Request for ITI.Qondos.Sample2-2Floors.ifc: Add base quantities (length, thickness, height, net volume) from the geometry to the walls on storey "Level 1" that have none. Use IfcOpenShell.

First a look at what the model holds.

```python
import ifcopenshell
import ifcopenshell.util.element
import ifcopenshell.util.unit

model = ifcopenshell.open("ITI.Qondos.Sample2-2Floors.ifc")
print(model.schema)
for unit_type in ("LENGTHUNIT", "AREAUNIT", "VOLUMEUNIT"):
    print(unit_type, ifcopenshell.util.unit.calculate_unit_scale(model, unit_type))
storey = next(s for s in model.by_type("IfcBuildingStorey") if s.Name == "Level 1")
walls = [e for e in ifcopenshell.util.element.get_decomposition(storey) if e.is_a("IfcWall")]
for e in sorted(walls, key=lambda e: e.id()):
    print(e.id(), e.is_a(), e.Name, list(ifcopenshell.util.element.get_psets(e, qtos_only=True)), sep=" | ")
```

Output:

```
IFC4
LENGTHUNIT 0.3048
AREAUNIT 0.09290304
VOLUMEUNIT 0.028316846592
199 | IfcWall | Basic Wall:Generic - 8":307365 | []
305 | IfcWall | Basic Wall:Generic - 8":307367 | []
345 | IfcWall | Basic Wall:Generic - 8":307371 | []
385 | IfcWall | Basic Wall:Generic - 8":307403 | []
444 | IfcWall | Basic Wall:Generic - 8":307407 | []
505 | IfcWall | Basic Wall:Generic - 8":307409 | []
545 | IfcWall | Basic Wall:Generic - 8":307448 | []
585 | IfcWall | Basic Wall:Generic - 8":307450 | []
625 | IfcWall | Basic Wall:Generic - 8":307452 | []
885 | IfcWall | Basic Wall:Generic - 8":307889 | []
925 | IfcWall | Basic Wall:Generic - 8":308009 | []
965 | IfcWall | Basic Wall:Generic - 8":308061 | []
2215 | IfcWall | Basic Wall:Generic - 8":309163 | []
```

```python
import ifcopenshell
import ifcopenshell.api.pset
import ifcopenshell.geom
import ifcopenshell.util.element
import ifcopenshell.util.shape
import ifcopenshell.util.unit

model = ifcopenshell.open("ITI.Qondos.Sample2-2Floors.ifc")
unit_scale = ifcopenshell.util.unit.calculate_unit_scale(model)
volume_scale = ifcopenshell.util.unit.calculate_unit_scale(model, "VOLUMEUNIT")
settings = ifcopenshell.geom.settings()

storey = next(s for s in model.by_type("IfcBuildingStorey") if s.Name == "Level 1")
walls = [e for e in ifcopenshell.util.element.get_decomposition(storey) if e.is_a("IfcWall")]

for e in sorted(walls, key=lambda e: e.id()):
    if ifcopenshell.util.element.get_psets(e, qtos_only=True, should_inherit=False):
        continue
    # Geometry comes back in metres, in the element's own axes.
    shape = ifcopenshell.geom.create_shape(settings, e)
    values = {
        "Length": ifcopenshell.util.shape.get_x(shape.geometry) / unit_scale,
        "Width": ifcopenshell.util.shape.get_y(shape.geometry) / unit_scale,
        "Height": ifcopenshell.util.shape.get_z(shape.geometry) / unit_scale,
        "NetVolume": ifcopenshell.util.shape.get_volume(shape.geometry) / volume_scale,
    }
    qto = ifcopenshell.api.pset.add_qto(model, product=e, name="Qto_WallBaseQuantities")
    ifcopenshell.api.pset.edit_qto(model, qto=qto, properties=values)
    print(e.id(), {k: round(v, 3) for k, v in values.items()})

model.write("ITI.Qondos.Sample2-2Floors_edited.ifc")
```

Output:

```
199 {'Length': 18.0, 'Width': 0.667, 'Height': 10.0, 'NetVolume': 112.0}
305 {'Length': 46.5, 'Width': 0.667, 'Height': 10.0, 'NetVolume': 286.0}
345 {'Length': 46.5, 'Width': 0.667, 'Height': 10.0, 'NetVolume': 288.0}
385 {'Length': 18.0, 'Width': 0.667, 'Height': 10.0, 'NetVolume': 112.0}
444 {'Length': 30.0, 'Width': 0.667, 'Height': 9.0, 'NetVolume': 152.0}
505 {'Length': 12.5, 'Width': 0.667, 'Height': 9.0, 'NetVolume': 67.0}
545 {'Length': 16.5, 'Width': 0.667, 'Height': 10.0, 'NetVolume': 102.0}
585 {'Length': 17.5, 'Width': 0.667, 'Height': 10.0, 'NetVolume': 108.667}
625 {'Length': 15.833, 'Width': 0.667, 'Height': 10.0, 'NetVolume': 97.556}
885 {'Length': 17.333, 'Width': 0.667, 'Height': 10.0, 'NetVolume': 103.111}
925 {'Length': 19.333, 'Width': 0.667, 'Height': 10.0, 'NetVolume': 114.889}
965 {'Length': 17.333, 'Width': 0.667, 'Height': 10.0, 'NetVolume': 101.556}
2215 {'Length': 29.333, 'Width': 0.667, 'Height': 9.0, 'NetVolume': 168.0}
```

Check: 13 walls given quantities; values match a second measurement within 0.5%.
